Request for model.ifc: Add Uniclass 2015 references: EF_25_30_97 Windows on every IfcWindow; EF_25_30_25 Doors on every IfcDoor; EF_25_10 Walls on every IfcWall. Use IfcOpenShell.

First a look at what the model holds.

```python
import ifcopenshell

model = ifcopenshell.open("model.ifc")
print(model.schema)
print("classifications:", [c.Name for c in model.by_type("IfcClassification")])
for ifc_class in ("IfcDoor", "IfcRoof", "IfcStair", "IfcWall", "IfcWindow"):
    print(ifc_class, len(model.by_type(ifc_class)))
```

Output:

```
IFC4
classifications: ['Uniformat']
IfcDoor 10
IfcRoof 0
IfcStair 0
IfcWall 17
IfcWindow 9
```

```python
import ifcopenshell
import ifcopenshell.api.classification

model = ifcopenshell.open("model.ifc")

system = ifcopenshell.api.classification.add_classification(model, classification="Uniclass 2015")

codes = {
    "IfcWindow": ("EF_25_30_97", "Windows"),
    "IfcDoor": ("EF_25_30_25", "Doors"),
    "IfcWall": ("EF_25_10", "Walls"),
}
for ifc_class, (code, name) in codes.items():
    products = model.by_type(ifc_class)
    ifcopenshell.api.classification.add_reference(
        model, products=products, classification=system, identification=code, name=name
    )
    print(code, len(products))

model.write("model_edited.ifc")
```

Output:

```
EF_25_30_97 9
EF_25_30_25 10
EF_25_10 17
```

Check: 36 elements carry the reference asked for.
